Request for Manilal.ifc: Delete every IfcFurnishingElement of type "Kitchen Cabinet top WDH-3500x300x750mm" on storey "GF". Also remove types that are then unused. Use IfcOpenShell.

First a look at what the model holds.

```python
import ifcopenshell
import ifcopenshell.util.element

model = ifcopenshell.open("Manilal.ifc")
print(model.schema)
storey = next(s for s in model.by_type("IfcBuildingStorey") if s.Name == "GF")
furniture = [e for e in ifcopenshell.util.element.get_decomposition(storey) if e.is_a("IfcFurnishingElement")]
seen = {}
for e in furniture:
    element_type = ifcopenshell.util.element.get_type(e)
    name = element_type.Name if element_type not in (None, e) else None
    seen[name] = seen.get(name, 0) + 1
for name, count in sorted(seen.items(), key=str):
    print(count, "x", name)
```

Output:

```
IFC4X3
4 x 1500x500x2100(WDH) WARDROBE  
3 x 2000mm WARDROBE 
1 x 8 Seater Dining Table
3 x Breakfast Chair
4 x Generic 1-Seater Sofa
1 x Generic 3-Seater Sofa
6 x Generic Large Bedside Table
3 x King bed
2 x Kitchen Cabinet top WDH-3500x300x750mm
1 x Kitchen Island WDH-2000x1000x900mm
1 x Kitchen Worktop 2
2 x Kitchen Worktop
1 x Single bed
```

```python
import ifcopenshell
import ifcopenshell.api.root
import ifcopenshell.util.element

model = ifcopenshell.open("Manilal.ifc")

storey = next(s for s in model.by_type("IfcBuildingStorey") if s.Name == "GF")
furniture = [e for e in ifcopenshell.util.element.get_decomposition(storey) if e.is_a("IfcFurnishingElement")]
targets = [e for e in furniture if (t := ifcopenshell.util.element.get_type(e)) not in (None, e) and t.Name == "Kitchen Cabinet top WDH-3500x300x750mm"]
types = {ifcopenshell.util.element.get_type(e) for e in targets} - {None, *targets}

for e in targets:
    ifcopenshell.api.root.remove_product(model, product=e)
print(len(targets), "removed")

unused = [t for t in types if not ifcopenshell.util.element.get_types(t)]
for t in unused:
    ifcopenshell.api.root.remove_product(model, product=t)
print(len(unused), "unused types removed")

model.write("Manilal-out.ifc")
```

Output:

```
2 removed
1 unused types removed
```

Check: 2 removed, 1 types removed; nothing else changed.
